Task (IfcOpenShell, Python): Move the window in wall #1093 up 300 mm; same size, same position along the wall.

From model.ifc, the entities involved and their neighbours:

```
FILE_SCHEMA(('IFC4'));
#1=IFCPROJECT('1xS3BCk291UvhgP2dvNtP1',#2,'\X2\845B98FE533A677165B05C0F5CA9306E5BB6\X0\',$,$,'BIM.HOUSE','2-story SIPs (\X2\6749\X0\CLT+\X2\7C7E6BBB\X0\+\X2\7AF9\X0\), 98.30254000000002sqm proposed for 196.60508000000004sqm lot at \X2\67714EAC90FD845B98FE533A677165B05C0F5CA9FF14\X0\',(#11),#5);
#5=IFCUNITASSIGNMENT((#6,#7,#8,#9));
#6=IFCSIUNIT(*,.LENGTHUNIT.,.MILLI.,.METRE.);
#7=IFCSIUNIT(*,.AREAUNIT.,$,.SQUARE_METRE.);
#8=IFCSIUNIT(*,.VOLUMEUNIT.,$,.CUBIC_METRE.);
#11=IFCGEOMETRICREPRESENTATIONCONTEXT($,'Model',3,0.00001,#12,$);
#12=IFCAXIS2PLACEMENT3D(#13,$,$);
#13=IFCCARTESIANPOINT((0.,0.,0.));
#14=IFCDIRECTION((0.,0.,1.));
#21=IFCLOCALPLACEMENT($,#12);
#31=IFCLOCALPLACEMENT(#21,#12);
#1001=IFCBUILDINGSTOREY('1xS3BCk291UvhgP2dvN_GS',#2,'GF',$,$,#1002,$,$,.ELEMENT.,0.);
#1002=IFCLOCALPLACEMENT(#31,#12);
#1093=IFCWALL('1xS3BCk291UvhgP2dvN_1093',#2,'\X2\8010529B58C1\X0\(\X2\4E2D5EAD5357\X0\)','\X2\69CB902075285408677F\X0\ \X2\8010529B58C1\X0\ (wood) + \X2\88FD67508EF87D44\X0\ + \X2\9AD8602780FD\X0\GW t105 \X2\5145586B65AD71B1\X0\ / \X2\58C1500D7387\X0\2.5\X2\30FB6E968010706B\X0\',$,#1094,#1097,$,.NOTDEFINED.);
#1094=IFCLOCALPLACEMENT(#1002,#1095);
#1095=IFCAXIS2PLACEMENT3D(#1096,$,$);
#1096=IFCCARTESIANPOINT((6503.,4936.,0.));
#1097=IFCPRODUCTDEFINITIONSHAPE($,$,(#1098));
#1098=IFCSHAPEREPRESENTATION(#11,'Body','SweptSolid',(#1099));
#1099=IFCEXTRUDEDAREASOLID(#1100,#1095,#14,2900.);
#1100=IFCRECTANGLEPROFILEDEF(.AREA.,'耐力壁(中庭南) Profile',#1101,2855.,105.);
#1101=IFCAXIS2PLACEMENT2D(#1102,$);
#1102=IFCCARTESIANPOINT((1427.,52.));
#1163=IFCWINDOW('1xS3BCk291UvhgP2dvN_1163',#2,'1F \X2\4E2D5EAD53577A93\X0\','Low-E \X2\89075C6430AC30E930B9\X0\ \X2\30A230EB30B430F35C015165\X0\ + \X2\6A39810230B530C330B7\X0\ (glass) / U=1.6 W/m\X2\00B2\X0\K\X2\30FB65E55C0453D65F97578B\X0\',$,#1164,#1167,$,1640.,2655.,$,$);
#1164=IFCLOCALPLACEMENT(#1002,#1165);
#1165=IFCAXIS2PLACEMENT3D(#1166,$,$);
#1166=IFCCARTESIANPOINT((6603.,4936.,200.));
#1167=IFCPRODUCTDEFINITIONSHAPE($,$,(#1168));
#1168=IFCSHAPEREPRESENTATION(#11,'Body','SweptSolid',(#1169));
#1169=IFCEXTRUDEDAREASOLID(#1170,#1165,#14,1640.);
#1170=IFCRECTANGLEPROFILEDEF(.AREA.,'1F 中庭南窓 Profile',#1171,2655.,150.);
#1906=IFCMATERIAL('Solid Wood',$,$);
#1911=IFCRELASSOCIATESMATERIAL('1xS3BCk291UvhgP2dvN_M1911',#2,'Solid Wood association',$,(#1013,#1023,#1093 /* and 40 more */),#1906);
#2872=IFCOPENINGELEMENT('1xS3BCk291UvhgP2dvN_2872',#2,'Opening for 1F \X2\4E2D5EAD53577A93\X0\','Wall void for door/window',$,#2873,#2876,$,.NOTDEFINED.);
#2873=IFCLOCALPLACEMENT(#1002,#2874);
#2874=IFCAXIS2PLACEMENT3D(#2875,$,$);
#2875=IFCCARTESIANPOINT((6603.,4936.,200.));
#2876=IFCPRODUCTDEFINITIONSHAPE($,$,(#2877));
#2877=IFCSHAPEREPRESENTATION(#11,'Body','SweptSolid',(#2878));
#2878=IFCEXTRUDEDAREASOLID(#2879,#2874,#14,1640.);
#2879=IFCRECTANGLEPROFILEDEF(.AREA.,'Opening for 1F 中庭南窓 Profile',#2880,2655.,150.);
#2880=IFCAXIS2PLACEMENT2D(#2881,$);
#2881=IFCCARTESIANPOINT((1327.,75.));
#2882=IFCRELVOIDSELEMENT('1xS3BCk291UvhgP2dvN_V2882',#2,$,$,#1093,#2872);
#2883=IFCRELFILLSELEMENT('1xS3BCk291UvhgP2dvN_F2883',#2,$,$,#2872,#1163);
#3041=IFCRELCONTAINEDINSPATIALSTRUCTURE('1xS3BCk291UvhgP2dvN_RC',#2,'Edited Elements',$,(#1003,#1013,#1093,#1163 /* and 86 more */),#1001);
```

```python
import numpy as np
import ifcopenshell
import ifcopenshell.api.geometry
import ifcopenshell.util.placement
import ifcopenshell.util.unit

model = ifcopenshell.open("model.ifc")
unit_scale = ifcopenshell.util.unit.calculate_unit_scale(model)

window = model.by_id(1163)
opening = window.FillsVoids[0].RelatingOpeningElement
dz = 300.0

shift = np.array([0.0, 0.0, dz])
# The window is not placed relative to its opening, so move both.
for product in (opening, window):
    matrix = ifcopenshell.util.placement.get_local_placement(product.ObjectPlacement)
    matrix[:3, 3] += shift
    ifcopenshell.api.geometry.edit_object_placement(model, product=product, matrix=matrix, is_si=False)

print(f"moved by {dz * unit_scale:+.3f} m")

model.write("model_rev.ifc")
```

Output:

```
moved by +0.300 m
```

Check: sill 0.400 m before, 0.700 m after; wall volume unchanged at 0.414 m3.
